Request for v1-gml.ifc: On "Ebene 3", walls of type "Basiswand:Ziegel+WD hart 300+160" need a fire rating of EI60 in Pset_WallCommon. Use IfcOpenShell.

First a look at what the model holds.

```python
import ifcopenshell
import ifcopenshell.util.element

model = ifcopenshell.open("v1-gml.ifc")
print(model.schema)
storey = next(s for s in model.by_type("IfcBuildingStorey") if s.Name == "Ebene 3")
walls = [e for e in ifcopenshell.util.element.get_decomposition(storey) if e.is_a("IfcWall")]
seen = {}
for e in walls:
    element_type = ifcopenshell.util.element.get_type(e)
    key = (element_type.Name if element_type != e and element_type else None, ifcopenshell.util.element.get_pset(e, "Pset_WallCommon", "FireRating"))
    seen[key] = seen.get(key, 0) + 1
for (name, value), count in sorted(seen.items(), key=str):
    print(count, "x", name, "|", value)
```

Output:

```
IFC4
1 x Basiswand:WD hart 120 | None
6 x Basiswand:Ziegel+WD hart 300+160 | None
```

```python
import ifcopenshell
import ifcopenshell.api.pset
import ifcopenshell.util.element

model = ifcopenshell.open("v1-gml.ifc")

storey = next(s for s in model.by_type("IfcBuildingStorey") if s.Name == "Ebene 3")
walls = [e for e in ifcopenshell.util.element.get_decomposition(storey) if e.is_a("IfcWall")]

count = 0
for e in walls:
    element_type = ifcopenshell.util.element.get_type(e)
    if element_type in (None, e) or element_type.Name != "Basiswand:Ziegel+WD hart 300+160":
        continue
    # add_pset returns the element's existing set when there is one.
    pset = ifcopenshell.api.pset.add_pset(model, product=e, name="Pset_WallCommon")
    ifcopenshell.api.pset.edit_pset(model, pset=pset, properties={"FireRating": "EI60"})
    count += 1

print(count, "walls updated")

model.write("v1-gml_rev.ifc")
```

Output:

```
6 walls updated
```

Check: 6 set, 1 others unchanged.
